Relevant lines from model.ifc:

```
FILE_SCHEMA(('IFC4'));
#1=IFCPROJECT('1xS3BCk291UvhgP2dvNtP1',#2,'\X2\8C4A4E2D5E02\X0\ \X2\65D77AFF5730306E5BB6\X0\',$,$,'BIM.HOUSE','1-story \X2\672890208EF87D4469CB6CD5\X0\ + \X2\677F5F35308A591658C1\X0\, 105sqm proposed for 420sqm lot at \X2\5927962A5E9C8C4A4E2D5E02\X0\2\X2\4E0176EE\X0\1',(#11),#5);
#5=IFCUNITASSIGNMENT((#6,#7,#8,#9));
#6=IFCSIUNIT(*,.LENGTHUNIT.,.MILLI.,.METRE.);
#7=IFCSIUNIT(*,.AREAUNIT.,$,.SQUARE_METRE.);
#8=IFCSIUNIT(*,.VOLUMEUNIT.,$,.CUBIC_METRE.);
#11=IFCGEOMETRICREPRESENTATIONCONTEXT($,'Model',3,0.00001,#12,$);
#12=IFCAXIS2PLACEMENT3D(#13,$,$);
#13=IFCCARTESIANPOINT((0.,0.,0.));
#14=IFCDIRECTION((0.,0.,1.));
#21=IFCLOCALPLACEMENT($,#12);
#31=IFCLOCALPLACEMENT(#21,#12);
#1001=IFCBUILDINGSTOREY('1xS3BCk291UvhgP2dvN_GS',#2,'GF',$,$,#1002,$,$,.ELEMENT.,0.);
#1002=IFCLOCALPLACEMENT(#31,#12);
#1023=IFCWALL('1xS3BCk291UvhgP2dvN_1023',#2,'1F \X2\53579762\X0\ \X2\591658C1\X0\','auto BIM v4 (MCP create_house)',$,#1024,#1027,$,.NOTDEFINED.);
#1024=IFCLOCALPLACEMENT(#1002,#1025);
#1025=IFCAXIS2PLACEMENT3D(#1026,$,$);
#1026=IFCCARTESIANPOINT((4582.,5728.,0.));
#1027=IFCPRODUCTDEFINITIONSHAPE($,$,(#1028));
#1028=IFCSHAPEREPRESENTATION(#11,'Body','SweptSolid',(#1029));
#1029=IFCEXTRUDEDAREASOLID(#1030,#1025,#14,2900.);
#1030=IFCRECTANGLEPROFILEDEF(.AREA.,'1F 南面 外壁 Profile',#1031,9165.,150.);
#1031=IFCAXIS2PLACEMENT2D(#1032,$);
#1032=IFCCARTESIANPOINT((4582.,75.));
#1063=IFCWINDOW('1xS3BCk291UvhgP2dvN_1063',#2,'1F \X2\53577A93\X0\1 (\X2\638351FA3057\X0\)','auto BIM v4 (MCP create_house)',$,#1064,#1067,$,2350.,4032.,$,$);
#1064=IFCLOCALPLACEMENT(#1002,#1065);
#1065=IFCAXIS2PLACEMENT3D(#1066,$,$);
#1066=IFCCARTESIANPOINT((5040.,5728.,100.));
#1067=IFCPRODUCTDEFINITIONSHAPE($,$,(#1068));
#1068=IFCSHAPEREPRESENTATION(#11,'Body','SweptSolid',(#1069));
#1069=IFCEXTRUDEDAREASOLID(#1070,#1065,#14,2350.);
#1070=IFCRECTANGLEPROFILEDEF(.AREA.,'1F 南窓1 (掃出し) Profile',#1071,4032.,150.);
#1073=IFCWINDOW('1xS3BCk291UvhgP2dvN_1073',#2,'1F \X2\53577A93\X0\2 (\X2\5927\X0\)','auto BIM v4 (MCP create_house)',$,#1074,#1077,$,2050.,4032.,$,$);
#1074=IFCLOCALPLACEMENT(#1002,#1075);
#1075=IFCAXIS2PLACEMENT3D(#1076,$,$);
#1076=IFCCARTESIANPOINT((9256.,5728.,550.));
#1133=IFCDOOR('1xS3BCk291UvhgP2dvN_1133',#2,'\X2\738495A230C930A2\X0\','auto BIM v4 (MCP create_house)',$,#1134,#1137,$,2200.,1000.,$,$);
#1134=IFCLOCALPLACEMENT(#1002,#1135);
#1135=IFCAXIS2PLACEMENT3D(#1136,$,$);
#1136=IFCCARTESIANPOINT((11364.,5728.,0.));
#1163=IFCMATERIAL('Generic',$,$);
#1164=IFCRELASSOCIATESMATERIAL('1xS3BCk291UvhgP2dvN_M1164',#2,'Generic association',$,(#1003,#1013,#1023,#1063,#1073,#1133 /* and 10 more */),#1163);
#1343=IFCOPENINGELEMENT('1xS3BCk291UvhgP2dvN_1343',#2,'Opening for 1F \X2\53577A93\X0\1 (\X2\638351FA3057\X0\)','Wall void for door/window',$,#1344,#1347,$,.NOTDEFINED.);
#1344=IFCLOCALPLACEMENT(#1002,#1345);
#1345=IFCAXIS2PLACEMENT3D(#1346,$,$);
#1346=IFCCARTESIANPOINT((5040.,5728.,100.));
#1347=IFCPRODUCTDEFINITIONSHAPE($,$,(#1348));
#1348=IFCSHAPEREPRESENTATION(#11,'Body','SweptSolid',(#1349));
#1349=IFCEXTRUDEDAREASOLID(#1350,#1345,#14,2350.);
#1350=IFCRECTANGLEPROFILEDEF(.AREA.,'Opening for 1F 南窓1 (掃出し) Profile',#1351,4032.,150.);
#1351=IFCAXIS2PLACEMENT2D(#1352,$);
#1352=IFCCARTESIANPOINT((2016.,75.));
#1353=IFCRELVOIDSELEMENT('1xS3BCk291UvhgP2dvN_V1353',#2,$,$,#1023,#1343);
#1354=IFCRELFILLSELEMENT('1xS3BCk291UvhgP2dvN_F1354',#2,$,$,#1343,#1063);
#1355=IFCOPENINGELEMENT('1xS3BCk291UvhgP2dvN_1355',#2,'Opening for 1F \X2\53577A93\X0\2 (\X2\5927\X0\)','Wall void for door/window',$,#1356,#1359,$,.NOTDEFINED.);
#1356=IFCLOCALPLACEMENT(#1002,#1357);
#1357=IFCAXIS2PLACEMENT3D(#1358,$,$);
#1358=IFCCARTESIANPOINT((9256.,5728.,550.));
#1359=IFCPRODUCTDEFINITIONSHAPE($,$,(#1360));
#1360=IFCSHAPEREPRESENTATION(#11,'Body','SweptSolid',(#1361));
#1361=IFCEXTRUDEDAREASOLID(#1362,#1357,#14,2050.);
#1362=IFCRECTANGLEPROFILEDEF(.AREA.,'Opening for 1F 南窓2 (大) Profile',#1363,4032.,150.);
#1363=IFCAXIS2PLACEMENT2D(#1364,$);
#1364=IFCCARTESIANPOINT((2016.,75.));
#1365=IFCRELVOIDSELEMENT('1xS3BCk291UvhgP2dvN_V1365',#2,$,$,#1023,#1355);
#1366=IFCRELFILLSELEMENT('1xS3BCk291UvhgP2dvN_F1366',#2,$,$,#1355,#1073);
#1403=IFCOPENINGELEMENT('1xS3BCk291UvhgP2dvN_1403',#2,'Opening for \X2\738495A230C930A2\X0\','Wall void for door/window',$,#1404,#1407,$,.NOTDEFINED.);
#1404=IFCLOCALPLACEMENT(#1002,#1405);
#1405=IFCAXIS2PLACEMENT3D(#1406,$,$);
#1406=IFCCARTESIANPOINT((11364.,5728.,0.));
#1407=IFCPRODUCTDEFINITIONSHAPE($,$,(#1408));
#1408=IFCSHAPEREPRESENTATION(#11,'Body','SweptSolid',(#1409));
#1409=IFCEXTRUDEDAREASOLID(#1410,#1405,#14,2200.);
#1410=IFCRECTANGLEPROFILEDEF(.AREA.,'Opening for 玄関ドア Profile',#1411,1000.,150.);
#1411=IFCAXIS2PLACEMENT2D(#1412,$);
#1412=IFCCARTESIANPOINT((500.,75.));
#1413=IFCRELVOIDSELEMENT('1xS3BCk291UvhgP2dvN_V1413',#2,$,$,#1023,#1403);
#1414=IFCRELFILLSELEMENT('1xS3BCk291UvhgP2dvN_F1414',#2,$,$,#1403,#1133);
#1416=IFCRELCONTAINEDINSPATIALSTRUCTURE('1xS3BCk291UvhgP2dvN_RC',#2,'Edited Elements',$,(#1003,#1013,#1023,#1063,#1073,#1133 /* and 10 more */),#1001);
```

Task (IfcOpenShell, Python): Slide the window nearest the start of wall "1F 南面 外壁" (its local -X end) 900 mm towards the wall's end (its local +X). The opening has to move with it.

```python
import ifcopenshell
import ifcopenshell.api.geometry
import ifcopenshell.util.placement
import ifcopenshell.util.unit

model = ifcopenshell.open("model.ifc")
unit_scale = ifcopenshell.util.unit.calculate_unit_scale(model)

window = model.by_id(1063)
opening = window.FillsVoids[0].RelatingOpeningElement
wall = opening.VoidsElements[0].RelatingBuildingElement

wall_matrix = ifcopenshell.util.placement.get_local_placement(wall.ObjectPlacement)
shift = wall_matrix[:3, 0] * 0.9 / unit_scale
before = ifcopenshell.util.placement.get_local_placement(window.ObjectPlacement)[:3, 3].copy()

# The window is not placed relative to its opening, so move both.
for product in (opening, window):
    matrix = ifcopenshell.util.placement.get_local_placement(product.ObjectPlacement)
    matrix[:3, 3] += shift
    ifcopenshell.api.geometry.edit_object_placement(model, product=product, matrix=matrix, is_si=False)

after = ifcopenshell.util.placement.get_local_placement(window.ObjectPlacement)[:3, 3]
print("window moved by", (after - before).round(3) + 0.0)

model.write("model_rev.ifc")
```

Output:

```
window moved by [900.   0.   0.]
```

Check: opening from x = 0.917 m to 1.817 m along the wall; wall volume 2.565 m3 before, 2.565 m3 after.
